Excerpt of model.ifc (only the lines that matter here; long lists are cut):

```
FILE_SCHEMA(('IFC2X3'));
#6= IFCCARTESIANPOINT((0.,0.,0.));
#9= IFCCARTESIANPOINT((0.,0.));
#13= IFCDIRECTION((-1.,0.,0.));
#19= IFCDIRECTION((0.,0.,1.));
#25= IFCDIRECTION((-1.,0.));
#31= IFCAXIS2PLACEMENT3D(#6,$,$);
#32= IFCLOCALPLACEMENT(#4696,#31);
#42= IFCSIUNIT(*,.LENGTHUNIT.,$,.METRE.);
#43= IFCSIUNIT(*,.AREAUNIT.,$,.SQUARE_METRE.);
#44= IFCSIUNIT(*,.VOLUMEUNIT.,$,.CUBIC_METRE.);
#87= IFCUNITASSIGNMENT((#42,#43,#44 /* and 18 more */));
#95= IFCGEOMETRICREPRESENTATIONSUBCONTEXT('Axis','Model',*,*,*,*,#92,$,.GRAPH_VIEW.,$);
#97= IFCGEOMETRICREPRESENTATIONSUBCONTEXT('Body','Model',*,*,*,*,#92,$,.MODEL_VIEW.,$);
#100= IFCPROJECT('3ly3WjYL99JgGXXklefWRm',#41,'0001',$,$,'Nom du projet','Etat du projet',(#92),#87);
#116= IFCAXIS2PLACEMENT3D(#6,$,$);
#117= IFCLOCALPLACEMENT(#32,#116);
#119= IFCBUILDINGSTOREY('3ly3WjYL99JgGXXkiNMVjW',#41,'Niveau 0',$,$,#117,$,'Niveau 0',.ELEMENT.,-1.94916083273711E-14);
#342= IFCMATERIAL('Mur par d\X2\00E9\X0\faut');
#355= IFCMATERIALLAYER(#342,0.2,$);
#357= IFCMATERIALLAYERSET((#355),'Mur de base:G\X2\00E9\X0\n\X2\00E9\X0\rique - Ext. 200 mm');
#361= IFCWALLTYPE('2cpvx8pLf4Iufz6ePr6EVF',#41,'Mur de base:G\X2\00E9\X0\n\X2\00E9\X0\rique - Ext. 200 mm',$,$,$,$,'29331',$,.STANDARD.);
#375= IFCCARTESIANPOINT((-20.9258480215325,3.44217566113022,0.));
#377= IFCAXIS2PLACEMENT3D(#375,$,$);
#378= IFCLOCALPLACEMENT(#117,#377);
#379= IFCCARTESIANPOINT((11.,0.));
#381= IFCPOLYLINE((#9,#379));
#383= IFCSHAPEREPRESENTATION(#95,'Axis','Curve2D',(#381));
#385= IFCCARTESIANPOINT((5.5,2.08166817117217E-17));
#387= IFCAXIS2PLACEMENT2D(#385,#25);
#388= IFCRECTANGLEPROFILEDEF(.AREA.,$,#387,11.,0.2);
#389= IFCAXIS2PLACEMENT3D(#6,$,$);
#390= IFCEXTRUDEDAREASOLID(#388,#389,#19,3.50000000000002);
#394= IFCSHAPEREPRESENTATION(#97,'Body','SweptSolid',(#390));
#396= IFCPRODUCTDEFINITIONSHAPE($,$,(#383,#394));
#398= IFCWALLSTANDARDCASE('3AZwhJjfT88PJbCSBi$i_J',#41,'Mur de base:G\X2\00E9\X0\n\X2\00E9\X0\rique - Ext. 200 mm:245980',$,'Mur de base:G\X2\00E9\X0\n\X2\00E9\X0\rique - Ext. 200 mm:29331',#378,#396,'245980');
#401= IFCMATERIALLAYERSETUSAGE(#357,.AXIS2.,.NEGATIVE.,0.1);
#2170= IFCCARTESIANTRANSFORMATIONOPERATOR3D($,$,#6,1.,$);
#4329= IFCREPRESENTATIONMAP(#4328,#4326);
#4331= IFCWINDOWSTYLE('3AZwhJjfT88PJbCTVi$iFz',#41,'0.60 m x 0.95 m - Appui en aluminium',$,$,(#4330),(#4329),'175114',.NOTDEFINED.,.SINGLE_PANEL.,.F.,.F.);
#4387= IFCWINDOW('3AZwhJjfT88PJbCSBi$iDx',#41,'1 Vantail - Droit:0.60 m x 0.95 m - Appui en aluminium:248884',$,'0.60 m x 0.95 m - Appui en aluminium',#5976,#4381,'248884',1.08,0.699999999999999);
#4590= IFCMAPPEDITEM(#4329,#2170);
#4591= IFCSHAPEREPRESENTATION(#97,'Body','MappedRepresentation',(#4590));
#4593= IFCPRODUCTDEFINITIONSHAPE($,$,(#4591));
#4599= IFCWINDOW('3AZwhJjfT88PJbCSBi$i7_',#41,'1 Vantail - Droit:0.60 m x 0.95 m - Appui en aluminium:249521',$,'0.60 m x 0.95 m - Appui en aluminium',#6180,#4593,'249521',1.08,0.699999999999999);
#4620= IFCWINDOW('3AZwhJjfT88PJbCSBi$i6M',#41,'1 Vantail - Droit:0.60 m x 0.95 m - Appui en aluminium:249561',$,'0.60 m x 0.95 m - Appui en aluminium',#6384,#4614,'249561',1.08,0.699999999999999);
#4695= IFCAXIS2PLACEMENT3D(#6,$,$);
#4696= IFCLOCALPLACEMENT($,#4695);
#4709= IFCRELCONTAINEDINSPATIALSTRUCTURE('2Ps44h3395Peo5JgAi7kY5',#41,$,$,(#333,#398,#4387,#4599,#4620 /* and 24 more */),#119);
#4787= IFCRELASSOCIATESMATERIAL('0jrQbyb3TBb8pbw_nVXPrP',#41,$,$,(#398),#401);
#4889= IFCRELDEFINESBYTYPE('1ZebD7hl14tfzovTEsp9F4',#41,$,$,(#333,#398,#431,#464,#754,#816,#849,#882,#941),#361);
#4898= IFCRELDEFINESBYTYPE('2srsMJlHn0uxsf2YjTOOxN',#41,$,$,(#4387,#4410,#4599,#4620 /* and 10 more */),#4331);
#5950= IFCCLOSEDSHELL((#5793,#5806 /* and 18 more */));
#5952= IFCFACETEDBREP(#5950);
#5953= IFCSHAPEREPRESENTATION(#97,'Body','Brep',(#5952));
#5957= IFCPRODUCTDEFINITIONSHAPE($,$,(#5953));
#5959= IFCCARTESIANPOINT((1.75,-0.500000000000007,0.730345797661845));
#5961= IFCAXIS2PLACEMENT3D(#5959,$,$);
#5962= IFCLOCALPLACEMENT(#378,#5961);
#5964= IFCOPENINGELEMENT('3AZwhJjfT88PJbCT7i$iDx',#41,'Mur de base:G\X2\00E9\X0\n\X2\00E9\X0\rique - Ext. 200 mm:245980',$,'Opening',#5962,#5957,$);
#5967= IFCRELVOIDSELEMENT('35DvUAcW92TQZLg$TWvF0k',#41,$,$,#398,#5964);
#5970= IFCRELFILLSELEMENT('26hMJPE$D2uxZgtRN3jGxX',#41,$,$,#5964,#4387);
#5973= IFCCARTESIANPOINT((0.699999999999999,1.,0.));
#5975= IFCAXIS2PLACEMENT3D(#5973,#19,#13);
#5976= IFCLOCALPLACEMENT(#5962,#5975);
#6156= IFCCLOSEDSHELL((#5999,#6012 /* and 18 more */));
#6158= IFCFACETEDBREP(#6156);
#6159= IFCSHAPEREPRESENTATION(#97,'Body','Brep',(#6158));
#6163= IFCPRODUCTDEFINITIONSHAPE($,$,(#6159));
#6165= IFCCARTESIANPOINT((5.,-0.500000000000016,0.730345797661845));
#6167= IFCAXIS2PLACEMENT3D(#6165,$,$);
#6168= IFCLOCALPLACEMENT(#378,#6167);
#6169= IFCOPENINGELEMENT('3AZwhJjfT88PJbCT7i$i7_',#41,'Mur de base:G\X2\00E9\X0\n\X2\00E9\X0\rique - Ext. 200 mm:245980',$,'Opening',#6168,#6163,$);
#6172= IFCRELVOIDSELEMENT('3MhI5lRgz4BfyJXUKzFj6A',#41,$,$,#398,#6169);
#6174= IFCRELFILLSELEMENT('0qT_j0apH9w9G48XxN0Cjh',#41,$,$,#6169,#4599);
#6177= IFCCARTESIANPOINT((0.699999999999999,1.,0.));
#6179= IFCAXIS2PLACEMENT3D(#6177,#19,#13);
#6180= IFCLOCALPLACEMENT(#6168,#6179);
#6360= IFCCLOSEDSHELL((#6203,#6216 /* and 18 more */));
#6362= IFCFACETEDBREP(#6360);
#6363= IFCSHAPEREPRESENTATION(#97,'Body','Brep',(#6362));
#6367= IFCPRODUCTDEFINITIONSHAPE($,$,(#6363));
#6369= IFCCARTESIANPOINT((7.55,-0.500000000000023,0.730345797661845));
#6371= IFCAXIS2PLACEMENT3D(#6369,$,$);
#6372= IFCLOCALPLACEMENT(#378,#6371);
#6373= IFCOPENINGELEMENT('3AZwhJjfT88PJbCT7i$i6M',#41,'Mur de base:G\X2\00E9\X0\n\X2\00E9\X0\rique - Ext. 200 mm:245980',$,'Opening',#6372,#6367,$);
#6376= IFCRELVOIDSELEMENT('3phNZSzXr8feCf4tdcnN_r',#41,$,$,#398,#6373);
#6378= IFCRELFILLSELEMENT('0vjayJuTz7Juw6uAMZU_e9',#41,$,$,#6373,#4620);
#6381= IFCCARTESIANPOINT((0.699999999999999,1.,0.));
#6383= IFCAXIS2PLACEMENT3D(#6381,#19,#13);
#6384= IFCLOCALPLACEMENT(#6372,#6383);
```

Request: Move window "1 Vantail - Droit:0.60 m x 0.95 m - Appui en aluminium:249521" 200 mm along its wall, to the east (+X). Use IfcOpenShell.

```python
import ifcopenshell
import ifcopenshell.api.geometry
import ifcopenshell.util.placement

model = ifcopenshell.open("model.ifc")

window = model.by_id(4599)
opening = window.FillsVoids[0].RelatingOpeningElement
wall = opening.VoidsElements[0].RelatingBuildingElement

wall_matrix = ifcopenshell.util.placement.get_local_placement(wall.ObjectPlacement)
shift = wall_matrix[:3, 0] * 0.2
before = ifcopenshell.util.placement.get_local_placement(window.ObjectPlacement)[:3, 3].copy()

# The window is placed relative to its opening, so it follows when the opening moves.
matrix = ifcopenshell.util.placement.get_local_placement(opening.ObjectPlacement)
matrix[:3, 3] += shift
ifcopenshell.api.geometry.edit_object_placement(
    model, product=opening, matrix=matrix, is_si=False, should_transform_children=True
)

after = ifcopenshell.util.placement.get_local_placement(window.ObjectPlacement)[:3, 3]
print("window moved by", (after - before).round(3) + 0.0)

model.write("model_v2.ifc")
```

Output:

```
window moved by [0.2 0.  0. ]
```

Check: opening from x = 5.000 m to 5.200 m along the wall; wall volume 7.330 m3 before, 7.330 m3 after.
